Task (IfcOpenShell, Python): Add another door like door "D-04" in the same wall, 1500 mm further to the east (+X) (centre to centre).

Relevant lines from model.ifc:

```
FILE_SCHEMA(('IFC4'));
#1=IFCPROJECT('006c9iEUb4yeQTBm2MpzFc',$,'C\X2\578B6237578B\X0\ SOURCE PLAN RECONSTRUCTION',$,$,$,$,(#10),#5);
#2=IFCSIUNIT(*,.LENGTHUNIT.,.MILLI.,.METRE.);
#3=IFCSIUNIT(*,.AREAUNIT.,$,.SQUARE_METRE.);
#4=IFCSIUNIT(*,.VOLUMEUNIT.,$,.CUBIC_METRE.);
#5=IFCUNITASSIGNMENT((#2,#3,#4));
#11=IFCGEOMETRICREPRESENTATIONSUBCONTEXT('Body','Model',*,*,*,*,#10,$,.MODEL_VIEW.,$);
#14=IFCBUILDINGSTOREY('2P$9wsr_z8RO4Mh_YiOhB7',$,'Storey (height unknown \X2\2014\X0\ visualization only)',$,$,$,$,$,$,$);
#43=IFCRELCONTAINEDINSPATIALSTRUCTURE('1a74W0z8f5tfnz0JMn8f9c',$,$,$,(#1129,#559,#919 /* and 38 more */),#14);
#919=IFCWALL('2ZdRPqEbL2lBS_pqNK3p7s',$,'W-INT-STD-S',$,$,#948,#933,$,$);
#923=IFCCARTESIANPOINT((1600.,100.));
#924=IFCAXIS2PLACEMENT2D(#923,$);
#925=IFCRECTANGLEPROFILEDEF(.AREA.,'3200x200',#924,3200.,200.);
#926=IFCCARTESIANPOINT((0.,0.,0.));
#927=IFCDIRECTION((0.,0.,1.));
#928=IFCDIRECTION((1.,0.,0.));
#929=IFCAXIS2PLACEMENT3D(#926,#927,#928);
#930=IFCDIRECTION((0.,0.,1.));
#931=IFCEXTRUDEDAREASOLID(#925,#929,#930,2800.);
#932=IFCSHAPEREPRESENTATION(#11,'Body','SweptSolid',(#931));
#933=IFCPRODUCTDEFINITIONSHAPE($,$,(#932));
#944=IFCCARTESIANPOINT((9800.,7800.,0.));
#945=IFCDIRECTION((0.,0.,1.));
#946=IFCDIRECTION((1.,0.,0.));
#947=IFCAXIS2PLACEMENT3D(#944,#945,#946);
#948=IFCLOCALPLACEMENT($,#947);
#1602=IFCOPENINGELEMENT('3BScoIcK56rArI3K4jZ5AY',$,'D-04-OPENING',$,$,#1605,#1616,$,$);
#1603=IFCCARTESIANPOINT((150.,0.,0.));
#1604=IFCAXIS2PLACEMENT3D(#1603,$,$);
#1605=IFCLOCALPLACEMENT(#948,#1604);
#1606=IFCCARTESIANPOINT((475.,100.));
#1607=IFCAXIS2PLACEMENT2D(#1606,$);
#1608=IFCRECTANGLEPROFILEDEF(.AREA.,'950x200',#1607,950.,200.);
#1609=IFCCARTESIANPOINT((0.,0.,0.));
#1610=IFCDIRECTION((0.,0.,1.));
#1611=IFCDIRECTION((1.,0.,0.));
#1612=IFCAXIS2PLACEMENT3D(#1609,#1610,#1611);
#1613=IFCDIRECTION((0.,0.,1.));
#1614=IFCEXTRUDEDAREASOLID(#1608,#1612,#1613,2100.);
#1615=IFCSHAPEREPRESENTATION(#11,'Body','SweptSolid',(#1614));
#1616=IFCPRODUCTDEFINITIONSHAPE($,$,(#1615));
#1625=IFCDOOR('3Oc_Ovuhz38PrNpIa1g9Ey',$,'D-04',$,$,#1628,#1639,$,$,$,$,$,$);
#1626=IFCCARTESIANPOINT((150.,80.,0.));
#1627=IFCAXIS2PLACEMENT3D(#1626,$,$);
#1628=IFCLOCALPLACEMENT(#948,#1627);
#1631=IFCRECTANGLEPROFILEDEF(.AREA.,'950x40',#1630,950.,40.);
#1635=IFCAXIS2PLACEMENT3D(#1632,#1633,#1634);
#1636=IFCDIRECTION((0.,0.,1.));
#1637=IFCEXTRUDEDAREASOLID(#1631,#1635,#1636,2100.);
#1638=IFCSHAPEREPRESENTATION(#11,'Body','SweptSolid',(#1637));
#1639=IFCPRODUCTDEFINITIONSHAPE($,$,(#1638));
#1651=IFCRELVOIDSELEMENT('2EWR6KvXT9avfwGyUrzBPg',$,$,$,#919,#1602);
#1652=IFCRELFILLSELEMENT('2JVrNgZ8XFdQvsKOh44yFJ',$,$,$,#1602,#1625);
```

```python
import ifcopenshell
import ifcopenshell.api.feature
import ifcopenshell.api.geometry
import ifcopenshell.api.root
import ifcopenshell.geom
import ifcopenshell.util.element
import ifcopenshell.util.placement
import ifcopenshell.util.shape

model = ifcopenshell.open("model.ifc")
settings = ifcopenshell.geom.settings()


def volume(element):
    """Net volume in cubic metres, openings subtracted."""
    shape = ifcopenshell.geom.create_shape(settings, element)
    return ifcopenshell.util.shape.get_volume(shape.geometry)


door = model.by_guid("3Oc_Ovuhz38PrNpIa1g9Ey")
opening = door.FillsVoids[0].RelatingOpeningElement
wall = opening.VoidsElements[0].RelatingBuildingElement
before = volume(wall)
shift = ifcopenshell.util.placement.get_local_placement(wall.ObjectPlacement)[:3, 0] * 1500.0

# copy_class copies the void relationship, type, container and properties, but no geometry.
new_opening = ifcopenshell.api.root.copy_class(model, product=opening)
new_opening.Representation = ifcopenshell.util.element.copy_deep(
    model, opening.Representation, exclude=["IfcGeometricRepresentationContext", "IfcRepresentationMap"]
)
new_door = ifcopenshell.api.root.copy_class(model, product=door)
new_door.Representation = ifcopenshell.util.element.copy_deep(
    model, door.Representation, exclude=["IfcGeometricRepresentationContext", "IfcRepresentationMap"]
)
ifcopenshell.api.feature.add_filling(model, opening=new_opening, element=new_door)

for old, new in ((opening, new_opening), (door, new_door)):
    matrix = ifcopenshell.util.placement.get_local_placement(old.ObjectPlacement)
    matrix[:3, 3] += shift
    ifcopenshell.api.geometry.edit_object_placement(model, product=new, matrix=matrix, is_si=False)

after = volume(wall)

print(f"wall volume {before:.3f} -> {after:.3f} m3")

model.write("model_edited.ifc")
```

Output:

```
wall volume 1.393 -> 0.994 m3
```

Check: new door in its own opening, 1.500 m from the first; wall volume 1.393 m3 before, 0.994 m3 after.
